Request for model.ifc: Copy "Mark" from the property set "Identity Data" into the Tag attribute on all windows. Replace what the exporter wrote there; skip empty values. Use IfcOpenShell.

First a look at what the model holds.

```python
import ifcopenshell
import ifcopenshell.util.element

model = ifcopenshell.open("model.ifc")
print(model.schema)
windows = model.by_type("IfcWindow")
print(len(windows), "windows")
for e in windows[:8]:
    source = ifcopenshell.util.element.get_pset(e, "Identity Data", "Mark")
    target = e.Tag
    print(e.id(), repr(source), repr(target), sep=" | ")
```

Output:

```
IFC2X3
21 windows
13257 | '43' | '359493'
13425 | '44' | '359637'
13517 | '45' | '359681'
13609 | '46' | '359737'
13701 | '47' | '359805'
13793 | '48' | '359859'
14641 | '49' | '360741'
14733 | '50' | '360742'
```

```python
import ifcopenshell
import ifcopenshell.util.element

model = ifcopenshell.open("model.ifc")

count = 0
for e in model.by_type("IfcWindow"):
    value = ifcopenshell.util.element.get_pset(e, "Identity Data", "Mark")
    current = e.Tag
    if not value or not value.strip() or current == value:
        continue
    e.Tag = value
    count += 1

print(count, "windows updated")

model.write("model_rev.ifc")
```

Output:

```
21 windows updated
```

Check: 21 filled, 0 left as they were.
